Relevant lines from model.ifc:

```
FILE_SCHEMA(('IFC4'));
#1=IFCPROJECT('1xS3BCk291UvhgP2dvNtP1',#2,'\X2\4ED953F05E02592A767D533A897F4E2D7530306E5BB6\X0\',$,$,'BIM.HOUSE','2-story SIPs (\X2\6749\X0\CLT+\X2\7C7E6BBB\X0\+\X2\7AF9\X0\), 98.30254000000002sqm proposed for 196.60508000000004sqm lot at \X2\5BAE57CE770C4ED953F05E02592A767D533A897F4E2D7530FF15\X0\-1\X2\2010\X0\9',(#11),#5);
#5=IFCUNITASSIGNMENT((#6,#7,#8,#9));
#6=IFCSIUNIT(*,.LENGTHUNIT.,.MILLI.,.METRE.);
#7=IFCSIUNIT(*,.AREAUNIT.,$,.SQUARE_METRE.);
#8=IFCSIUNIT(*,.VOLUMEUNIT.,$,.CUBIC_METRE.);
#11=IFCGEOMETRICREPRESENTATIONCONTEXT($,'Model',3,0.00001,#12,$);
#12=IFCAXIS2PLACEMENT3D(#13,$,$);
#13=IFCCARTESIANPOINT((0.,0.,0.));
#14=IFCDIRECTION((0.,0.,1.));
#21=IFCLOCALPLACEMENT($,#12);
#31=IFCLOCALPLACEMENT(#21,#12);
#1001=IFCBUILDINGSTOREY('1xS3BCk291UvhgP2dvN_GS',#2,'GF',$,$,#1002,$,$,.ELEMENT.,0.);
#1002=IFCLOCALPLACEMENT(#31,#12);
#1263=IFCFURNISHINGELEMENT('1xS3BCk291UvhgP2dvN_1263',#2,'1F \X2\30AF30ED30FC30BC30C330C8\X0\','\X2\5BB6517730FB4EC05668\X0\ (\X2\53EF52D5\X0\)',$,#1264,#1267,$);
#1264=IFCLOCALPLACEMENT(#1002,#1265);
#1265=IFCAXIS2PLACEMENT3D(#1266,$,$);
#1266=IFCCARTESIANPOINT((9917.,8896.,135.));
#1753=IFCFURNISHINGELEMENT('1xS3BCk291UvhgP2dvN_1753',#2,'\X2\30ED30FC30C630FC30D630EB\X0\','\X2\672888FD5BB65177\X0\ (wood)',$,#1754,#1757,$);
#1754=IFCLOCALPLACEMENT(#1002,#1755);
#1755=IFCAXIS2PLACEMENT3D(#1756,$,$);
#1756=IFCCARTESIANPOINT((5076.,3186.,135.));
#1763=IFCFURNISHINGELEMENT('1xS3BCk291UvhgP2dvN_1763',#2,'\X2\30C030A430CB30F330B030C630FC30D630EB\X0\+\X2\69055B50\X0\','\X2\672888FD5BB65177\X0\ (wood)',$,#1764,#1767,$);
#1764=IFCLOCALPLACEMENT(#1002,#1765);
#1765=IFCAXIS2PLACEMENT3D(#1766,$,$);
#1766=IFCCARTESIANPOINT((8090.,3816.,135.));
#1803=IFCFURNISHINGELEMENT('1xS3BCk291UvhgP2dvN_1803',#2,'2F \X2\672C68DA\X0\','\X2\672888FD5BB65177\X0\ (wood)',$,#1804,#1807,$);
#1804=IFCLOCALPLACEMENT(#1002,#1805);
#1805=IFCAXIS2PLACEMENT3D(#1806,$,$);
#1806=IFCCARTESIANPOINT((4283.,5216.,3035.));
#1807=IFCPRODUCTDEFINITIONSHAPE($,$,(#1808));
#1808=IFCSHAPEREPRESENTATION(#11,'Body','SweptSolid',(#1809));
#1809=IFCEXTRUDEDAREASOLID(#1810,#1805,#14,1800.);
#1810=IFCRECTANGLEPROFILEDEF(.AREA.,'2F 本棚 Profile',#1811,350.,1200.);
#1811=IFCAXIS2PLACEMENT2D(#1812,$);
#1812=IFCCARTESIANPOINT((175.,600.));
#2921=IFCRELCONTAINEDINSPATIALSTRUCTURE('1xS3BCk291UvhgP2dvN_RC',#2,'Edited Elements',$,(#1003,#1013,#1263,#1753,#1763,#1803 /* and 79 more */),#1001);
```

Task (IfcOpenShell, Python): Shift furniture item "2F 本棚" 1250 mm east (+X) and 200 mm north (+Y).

```python
import ifcopenshell
import ifcopenshell.api.geometry
import ifcopenshell.util.placement
import ifcopenshell.util.unit

model = ifcopenshell.open("model.ifc")
unit_scale = ifcopenshell.util.unit.calculate_unit_scale(model)

item = model.by_guid("1xS3BCk291UvhgP2dvN_1803")
matrix = ifcopenshell.util.placement.get_local_placement(item.ObjectPlacement)
matrix[0, 3] += 1.25 / unit_scale
matrix[1, 3] += 0.2 / unit_scale
ifcopenshell.api.geometry.edit_object_placement(model, product=item, matrix=matrix, is_si=False)

print(ifcopenshell.util.placement.get_local_placement(item.ObjectPlacement).round(3) + 0.0)

model.write("model-out.ifc")
```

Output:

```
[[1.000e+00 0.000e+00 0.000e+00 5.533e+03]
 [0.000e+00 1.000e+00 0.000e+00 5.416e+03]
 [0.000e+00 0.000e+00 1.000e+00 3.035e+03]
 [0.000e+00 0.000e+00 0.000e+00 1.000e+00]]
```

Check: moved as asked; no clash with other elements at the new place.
